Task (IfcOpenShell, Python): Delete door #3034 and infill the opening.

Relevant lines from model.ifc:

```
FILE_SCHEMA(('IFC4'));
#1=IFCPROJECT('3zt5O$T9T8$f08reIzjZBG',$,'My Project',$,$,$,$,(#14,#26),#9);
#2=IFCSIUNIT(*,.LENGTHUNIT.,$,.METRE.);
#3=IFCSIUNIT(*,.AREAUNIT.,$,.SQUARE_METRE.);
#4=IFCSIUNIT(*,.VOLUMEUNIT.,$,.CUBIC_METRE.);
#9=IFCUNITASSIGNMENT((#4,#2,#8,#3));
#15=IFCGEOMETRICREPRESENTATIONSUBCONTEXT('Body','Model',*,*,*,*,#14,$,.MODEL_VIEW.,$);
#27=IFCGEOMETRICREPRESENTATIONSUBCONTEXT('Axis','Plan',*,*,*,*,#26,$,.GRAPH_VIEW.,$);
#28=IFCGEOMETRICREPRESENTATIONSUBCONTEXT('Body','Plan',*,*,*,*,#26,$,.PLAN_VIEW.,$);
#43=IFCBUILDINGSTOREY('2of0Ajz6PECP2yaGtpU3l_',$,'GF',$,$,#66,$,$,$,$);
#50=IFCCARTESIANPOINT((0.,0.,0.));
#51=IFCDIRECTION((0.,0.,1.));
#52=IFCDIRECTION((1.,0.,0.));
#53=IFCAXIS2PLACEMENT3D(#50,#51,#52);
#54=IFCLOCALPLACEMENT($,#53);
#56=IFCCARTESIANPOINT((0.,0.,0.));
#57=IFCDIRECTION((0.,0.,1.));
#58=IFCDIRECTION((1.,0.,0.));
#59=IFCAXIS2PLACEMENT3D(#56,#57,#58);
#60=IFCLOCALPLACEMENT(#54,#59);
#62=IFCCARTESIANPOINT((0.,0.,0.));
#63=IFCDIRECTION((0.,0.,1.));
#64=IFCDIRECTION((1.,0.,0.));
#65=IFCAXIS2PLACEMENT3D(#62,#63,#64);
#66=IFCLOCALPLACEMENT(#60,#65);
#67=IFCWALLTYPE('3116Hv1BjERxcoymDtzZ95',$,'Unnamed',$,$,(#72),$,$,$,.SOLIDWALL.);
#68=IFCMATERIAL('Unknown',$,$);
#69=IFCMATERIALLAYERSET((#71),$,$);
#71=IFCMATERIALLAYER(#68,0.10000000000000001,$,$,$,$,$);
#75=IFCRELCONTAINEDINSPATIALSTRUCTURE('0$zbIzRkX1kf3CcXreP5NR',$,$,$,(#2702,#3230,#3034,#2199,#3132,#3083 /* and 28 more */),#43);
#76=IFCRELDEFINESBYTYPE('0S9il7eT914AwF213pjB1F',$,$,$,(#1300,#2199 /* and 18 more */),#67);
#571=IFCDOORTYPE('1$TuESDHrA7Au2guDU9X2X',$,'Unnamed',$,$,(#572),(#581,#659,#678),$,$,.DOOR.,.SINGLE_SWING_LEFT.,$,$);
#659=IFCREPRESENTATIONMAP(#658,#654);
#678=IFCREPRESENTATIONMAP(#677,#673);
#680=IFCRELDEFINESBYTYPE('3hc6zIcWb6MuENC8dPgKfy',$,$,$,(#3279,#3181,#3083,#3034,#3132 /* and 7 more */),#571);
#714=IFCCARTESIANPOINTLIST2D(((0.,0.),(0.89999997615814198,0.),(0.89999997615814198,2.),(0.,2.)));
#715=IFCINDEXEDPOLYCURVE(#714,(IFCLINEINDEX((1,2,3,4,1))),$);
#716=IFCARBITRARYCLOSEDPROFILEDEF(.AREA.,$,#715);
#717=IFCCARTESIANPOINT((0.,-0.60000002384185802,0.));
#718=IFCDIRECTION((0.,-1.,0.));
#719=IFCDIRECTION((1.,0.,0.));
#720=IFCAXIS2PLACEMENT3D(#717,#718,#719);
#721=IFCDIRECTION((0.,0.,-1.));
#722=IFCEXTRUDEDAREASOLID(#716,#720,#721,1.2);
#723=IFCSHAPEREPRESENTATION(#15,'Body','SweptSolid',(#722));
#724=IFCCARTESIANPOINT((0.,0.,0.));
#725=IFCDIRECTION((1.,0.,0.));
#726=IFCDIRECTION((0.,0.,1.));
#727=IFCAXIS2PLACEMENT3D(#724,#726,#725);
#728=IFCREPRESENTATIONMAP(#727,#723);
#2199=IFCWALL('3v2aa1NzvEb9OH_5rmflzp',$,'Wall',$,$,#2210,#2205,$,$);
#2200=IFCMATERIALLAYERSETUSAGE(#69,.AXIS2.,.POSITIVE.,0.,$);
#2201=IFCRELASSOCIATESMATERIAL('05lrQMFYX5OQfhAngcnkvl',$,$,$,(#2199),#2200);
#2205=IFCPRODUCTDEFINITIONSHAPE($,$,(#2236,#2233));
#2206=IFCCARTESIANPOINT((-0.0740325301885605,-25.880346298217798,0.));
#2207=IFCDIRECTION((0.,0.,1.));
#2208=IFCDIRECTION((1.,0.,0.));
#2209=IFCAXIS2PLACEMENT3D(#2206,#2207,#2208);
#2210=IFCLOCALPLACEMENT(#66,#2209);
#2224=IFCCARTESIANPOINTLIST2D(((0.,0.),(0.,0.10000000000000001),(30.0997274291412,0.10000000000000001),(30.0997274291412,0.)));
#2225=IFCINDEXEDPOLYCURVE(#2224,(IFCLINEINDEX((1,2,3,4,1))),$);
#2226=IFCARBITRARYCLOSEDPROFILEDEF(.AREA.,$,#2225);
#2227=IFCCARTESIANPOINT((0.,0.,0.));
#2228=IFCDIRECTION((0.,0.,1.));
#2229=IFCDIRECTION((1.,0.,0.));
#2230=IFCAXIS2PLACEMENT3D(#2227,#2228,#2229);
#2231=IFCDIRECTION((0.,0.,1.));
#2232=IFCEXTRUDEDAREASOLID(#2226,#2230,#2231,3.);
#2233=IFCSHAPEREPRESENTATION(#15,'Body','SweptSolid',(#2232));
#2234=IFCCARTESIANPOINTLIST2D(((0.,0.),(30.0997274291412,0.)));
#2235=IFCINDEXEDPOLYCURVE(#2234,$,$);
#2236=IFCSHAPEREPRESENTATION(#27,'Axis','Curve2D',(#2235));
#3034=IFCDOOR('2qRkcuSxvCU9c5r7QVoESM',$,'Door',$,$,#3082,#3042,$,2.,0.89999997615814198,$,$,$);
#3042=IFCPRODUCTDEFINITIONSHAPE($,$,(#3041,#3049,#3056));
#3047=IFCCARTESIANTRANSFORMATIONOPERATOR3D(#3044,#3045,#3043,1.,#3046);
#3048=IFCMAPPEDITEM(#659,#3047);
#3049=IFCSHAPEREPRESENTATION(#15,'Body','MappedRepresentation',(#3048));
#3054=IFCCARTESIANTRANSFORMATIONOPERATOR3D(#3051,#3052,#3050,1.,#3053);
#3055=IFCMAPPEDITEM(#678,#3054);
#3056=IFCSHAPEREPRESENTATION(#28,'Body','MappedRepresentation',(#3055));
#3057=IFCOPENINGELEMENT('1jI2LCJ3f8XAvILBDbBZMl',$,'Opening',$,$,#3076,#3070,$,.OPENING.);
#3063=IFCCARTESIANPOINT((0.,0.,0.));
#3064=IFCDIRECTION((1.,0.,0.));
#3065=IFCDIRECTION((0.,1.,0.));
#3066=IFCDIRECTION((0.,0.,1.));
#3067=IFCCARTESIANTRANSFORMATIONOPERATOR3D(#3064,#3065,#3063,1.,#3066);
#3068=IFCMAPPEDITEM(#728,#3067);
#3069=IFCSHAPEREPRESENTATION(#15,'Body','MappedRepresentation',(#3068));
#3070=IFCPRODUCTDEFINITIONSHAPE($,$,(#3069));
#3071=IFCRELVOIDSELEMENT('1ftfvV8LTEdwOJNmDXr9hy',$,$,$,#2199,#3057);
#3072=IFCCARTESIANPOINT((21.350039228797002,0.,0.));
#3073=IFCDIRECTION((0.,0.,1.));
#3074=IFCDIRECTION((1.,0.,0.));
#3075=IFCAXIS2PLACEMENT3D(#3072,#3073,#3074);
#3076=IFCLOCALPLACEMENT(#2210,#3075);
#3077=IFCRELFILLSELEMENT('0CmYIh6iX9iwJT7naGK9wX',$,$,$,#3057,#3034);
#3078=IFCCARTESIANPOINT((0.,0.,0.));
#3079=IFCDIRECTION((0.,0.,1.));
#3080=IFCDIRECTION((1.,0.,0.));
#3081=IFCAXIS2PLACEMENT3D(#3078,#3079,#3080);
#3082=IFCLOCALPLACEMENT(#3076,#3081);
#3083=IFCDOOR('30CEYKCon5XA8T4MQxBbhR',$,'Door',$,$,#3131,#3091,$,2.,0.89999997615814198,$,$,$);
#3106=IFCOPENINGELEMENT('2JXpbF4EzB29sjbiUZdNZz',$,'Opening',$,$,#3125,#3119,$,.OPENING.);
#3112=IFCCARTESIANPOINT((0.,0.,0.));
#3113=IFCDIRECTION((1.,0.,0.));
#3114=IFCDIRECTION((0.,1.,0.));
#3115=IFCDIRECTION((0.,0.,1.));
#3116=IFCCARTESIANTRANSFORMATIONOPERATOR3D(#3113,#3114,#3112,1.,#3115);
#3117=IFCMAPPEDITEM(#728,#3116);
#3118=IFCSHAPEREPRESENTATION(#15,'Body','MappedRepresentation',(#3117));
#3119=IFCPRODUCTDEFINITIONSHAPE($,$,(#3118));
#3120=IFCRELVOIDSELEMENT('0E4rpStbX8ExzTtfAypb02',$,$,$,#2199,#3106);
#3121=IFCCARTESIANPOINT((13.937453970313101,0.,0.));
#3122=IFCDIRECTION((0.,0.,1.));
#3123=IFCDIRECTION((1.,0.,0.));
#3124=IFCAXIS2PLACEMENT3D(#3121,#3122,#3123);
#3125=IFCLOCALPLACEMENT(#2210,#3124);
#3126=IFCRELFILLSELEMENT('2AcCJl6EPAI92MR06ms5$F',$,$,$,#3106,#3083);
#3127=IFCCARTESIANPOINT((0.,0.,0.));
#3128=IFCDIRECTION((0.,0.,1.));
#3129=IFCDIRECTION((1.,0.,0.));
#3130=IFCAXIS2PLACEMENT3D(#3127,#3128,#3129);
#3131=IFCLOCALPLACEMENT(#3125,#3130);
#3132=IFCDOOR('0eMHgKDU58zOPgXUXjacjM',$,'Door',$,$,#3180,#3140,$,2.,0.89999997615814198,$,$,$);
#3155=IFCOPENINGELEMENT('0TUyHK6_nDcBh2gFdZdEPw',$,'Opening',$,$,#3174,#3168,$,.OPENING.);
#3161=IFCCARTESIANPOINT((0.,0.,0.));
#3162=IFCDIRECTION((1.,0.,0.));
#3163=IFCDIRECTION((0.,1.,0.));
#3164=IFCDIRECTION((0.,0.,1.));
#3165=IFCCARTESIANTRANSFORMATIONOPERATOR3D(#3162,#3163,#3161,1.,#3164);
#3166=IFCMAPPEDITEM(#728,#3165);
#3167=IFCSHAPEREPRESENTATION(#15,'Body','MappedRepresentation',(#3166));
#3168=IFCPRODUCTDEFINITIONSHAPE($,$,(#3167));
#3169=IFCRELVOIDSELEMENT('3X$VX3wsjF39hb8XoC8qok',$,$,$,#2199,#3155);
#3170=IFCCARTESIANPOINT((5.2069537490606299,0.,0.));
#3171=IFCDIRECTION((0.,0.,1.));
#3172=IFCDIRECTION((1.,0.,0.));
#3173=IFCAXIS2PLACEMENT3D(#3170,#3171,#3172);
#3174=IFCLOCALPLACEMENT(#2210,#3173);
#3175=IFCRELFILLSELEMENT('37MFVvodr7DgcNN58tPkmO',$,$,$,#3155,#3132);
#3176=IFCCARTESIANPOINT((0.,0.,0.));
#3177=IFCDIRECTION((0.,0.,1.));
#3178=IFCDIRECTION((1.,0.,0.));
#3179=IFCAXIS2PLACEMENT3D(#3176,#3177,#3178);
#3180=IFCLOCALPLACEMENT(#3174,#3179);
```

```python
import ifcopenshell
import ifcopenshell.api.feature
import ifcopenshell.api.root
import ifcopenshell.geom
import ifcopenshell.util.shape

model = ifcopenshell.open("model.ifc")
settings = ifcopenshell.geom.settings()


def volume(element):
    """Net volume in cubic metres, openings subtracted."""
    shape = ifcopenshell.geom.create_shape(settings, element)
    return ifcopenshell.util.shape.get_volume(shape.geometry)


door = model.by_id(3034)
opening = door.FillsVoids[0].RelatingOpeningElement
wall = opening.VoidsElements[0].RelatingBuildingElement
before = volume(wall)

ifcopenshell.api.root.remove_product(model, product=door)
ifcopenshell.api.feature.remove_feature(model, feature=opening)

after = volume(wall)

print(f"wall volume {before:.3f} -> {after:.3f} m3")

model.write("model-out.ifc")
```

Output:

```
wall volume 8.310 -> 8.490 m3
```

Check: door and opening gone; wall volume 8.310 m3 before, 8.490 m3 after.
